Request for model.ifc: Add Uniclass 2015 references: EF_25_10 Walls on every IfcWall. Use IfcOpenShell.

First a look at what the model holds.

```python
import ifcopenshell

model = ifcopenshell.open("model.ifc")
print(model.schema)
print("classifications:", [c.Name for c in model.by_type("IfcClassification")])
for ifc_class in ("IfcDoor", "IfcRoof", "IfcStair", "IfcWall", "IfcWindow"):
    print(ifc_class, len(model.by_type(ifc_class)))
```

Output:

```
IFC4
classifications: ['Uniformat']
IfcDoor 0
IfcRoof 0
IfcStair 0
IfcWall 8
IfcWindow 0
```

```python
import ifcopenshell
import ifcopenshell.api.classification

model = ifcopenshell.open("model.ifc")

system = ifcopenshell.api.classification.add_classification(model, classification="Uniclass 2015")

codes = {
    "IfcWall": ("EF_25_10", "Walls"),
}
for ifc_class, (code, name) in codes.items():
    products = model.by_type(ifc_class)
    ifcopenshell.api.classification.add_reference(
        model, products=products, classification=system, identification=code, name=name
    )
    print(code, len(products))

model.write("model_v2.ifc")
```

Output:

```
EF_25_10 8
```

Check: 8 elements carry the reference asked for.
